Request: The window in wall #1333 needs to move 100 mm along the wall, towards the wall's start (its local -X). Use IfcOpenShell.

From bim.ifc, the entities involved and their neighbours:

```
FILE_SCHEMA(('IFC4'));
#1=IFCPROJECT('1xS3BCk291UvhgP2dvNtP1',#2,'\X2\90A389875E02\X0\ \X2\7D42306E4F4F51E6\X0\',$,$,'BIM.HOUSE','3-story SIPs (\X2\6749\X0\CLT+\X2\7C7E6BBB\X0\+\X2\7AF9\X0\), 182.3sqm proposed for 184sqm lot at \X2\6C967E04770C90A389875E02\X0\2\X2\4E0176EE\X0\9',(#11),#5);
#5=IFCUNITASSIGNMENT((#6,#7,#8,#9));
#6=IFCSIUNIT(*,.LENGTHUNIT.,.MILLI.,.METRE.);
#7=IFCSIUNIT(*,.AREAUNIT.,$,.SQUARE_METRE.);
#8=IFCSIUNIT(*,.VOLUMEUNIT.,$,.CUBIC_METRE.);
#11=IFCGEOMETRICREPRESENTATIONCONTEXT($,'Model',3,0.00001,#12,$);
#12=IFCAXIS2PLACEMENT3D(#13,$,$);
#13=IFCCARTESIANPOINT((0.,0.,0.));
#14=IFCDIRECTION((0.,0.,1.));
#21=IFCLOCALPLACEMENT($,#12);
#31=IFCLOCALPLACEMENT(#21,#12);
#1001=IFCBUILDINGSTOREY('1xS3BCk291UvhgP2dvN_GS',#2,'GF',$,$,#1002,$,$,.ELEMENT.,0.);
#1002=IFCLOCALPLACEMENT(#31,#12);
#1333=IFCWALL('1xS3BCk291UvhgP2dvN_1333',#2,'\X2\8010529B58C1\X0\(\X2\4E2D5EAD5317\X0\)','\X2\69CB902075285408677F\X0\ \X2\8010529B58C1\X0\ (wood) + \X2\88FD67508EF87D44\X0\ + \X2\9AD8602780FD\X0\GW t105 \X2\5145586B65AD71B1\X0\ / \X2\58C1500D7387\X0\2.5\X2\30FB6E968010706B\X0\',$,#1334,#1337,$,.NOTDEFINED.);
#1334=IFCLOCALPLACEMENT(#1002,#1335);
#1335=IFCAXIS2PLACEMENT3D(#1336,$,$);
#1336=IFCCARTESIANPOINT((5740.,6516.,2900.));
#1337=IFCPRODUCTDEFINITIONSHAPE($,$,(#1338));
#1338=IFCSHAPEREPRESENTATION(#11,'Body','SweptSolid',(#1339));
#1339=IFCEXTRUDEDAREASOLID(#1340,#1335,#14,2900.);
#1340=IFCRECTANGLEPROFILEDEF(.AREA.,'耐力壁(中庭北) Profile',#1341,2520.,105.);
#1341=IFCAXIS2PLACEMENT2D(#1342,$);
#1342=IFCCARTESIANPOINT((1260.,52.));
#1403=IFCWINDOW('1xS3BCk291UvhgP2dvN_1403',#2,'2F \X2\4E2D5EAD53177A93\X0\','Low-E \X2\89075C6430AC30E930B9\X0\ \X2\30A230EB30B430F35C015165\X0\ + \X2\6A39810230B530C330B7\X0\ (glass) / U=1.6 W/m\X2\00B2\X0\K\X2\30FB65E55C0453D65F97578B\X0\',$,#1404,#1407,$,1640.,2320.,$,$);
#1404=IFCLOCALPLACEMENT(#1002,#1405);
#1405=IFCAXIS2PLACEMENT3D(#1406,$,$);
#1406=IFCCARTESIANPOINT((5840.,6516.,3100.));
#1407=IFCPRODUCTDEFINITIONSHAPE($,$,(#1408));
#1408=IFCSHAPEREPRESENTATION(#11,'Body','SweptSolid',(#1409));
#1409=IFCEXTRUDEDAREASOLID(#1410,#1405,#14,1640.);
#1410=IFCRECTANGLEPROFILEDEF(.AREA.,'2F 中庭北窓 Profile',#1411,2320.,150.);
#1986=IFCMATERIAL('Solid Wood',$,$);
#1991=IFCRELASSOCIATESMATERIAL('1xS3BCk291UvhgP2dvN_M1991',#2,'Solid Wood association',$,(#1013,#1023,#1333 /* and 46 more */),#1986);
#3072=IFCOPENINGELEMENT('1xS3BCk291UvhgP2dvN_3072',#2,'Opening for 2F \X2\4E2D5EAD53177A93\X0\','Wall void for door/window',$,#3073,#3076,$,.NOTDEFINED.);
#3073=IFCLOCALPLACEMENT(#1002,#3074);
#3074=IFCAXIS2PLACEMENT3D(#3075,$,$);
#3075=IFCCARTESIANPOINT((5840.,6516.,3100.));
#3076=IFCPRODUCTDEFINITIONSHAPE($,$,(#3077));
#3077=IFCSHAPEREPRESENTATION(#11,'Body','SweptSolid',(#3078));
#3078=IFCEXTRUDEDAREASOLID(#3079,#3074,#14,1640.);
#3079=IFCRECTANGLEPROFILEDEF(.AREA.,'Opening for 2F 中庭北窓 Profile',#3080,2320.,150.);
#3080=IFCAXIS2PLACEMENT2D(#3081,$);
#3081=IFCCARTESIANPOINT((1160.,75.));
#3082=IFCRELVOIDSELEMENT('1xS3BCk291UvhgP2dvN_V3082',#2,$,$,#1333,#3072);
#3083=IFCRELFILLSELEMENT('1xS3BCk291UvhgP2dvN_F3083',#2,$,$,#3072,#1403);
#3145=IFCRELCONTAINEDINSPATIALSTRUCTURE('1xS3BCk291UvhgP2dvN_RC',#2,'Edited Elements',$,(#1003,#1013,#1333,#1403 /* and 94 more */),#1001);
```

```python
import ifcopenshell
import ifcopenshell.api.geometry
import ifcopenshell.util.placement

model = ifcopenshell.open("bim.ifc")

window = model.by_id(1403)
opening = window.FillsVoids[0].RelatingOpeningElement
wall = opening.VoidsElements[0].RelatingBuildingElement

wall_matrix = ifcopenshell.util.placement.get_local_placement(wall.ObjectPlacement)
shift = wall_matrix[:3, 0] * -100.0
before = ifcopenshell.util.placement.get_local_placement(window.ObjectPlacement)[:3, 3].copy()

# The window is not placed relative to its opening, so move both.
for product in (opening, window):
    matrix = ifcopenshell.util.placement.get_local_placement(product.ObjectPlacement)
    matrix[:3, 3] += shift
    ifcopenshell.api.geometry.edit_object_placement(model, product=product, matrix=matrix, is_si=False)

after = ifcopenshell.util.placement.get_local_placement(window.ObjectPlacement)[:3, 3]
print("window moved by", (after - before).round(3) + 0.0)

model.write("bim_updated.ifc")
```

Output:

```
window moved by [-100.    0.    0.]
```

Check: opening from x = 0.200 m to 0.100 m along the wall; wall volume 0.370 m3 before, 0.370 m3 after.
